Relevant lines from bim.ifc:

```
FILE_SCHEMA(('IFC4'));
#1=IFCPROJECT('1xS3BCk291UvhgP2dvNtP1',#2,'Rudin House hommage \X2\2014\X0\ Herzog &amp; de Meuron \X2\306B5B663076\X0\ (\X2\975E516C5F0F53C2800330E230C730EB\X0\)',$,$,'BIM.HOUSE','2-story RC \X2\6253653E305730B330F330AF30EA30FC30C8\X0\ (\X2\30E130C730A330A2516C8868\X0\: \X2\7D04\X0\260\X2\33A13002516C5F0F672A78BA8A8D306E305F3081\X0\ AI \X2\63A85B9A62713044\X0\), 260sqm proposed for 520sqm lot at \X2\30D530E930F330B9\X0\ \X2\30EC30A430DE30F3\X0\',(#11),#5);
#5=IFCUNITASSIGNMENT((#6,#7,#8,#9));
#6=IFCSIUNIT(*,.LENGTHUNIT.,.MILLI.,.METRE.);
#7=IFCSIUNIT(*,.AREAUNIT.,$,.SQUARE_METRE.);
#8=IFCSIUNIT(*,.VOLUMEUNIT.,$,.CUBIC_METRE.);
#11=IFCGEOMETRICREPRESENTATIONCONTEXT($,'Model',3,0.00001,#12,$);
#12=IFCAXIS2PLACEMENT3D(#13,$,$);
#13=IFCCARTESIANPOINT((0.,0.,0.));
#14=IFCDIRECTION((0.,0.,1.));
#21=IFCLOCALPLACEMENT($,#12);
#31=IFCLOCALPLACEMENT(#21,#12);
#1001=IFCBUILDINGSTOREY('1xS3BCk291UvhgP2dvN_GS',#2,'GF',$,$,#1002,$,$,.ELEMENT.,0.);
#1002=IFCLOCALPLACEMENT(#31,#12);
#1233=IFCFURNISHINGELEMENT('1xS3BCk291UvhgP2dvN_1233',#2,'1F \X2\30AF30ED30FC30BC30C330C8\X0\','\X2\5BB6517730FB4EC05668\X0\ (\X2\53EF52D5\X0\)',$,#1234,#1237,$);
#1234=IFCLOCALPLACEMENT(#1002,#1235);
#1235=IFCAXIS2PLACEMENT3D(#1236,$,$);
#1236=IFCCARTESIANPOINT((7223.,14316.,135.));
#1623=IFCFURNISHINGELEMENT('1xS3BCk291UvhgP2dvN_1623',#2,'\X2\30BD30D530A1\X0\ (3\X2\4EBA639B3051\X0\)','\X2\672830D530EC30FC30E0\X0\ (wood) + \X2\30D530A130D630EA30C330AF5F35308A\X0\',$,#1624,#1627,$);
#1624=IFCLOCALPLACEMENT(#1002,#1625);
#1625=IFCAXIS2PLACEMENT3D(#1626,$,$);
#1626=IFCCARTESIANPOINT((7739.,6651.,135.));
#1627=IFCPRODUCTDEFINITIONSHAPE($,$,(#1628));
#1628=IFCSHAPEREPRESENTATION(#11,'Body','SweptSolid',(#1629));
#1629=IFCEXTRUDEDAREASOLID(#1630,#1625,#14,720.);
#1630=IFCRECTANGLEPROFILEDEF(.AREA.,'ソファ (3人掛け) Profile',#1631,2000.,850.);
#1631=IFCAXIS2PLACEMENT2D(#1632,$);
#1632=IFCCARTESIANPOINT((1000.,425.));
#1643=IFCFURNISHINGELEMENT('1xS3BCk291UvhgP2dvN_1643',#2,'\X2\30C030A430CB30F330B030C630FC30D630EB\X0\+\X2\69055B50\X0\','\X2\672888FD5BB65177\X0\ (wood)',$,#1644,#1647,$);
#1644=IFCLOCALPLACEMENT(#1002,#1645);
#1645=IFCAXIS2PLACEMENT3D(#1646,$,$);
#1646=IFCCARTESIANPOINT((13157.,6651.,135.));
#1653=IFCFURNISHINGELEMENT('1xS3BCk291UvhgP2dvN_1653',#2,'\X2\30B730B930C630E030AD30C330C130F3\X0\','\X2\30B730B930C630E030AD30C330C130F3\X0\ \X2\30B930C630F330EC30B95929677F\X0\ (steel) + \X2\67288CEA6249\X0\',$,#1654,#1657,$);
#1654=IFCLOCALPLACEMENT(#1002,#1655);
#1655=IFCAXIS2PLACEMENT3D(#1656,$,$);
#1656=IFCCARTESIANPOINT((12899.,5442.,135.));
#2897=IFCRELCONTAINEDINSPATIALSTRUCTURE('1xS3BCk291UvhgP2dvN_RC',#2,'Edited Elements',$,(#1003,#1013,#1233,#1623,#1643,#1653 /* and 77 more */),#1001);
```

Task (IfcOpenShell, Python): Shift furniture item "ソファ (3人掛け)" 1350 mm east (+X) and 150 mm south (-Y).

```python
import ifcopenshell
import ifcopenshell.api.geometry
import ifcopenshell.util.placement

model = ifcopenshell.open("bim.ifc")

item = model.by_id(1623)
matrix = ifcopenshell.util.placement.get_local_placement(item.ObjectPlacement)
matrix[0, 3] += 1350.0
matrix[1, 3] -= 150.0
ifcopenshell.api.geometry.edit_object_placement(model, product=item, matrix=matrix, is_si=False)

print(ifcopenshell.util.placement.get_local_placement(item.ObjectPlacement).round(3) + 0.0)

model.write("bim_v2.ifc")
```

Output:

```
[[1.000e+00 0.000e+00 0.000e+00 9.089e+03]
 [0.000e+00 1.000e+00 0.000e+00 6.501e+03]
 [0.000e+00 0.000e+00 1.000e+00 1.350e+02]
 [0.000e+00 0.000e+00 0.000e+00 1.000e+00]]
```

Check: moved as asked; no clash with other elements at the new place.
